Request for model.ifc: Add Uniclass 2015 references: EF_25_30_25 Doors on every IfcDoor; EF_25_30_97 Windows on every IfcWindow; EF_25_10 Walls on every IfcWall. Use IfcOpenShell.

First a look at what the model holds.

```python
import ifcopenshell

model = ifcopenshell.open("model.ifc")
print(model.schema)
print("classifications:", [c.Name for c in model.by_type("IfcClassification")])
for ifc_class in ("IfcDoor", "IfcRoof", "IfcStair", "IfcWall", "IfcWindow"):
    print(ifc_class, len(model.by_type(ifc_class)))
```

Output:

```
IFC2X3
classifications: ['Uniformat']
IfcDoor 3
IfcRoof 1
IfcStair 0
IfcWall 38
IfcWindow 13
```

```python
import ifcopenshell
import ifcopenshell.api.classification

model = ifcopenshell.open("model.ifc")

# IFC2X3 requires Source and Edition and has no link from the project to the system.
system = model.create_entity("IfcClassification", Source="NBS", Edition="2015", Name="Uniclass 2015")

codes = {
    "IfcDoor": ("EF_25_30_25", "Doors"),
    "IfcWindow": ("EF_25_30_97", "Windows"),
    "IfcWall": ("EF_25_10", "Walls"),
}
for ifc_class, (code, name) in codes.items():
    products = model.by_type(ifc_class)
    ifcopenshell.api.classification.add_reference(
        model, products=products, classification=system, identification=code, name=name
    )
    print(code, len(products))

model.write("model_v2.ifc")
```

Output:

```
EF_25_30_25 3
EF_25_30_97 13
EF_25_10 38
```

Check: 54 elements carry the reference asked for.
